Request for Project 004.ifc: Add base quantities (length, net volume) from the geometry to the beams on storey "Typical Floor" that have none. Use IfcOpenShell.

First a look at what the model holds.

```python
import ifcopenshell
import ifcopenshell.util.element
import ifcopenshell.util.unit

model = ifcopenshell.open("Project 004.ifc")
print(model.schema)
for unit_type in ("LENGTHUNIT", "AREAUNIT", "VOLUMEUNIT"):
    print(unit_type, ifcopenshell.util.unit.calculate_unit_scale(model, unit_type))
storey = next(s for s in model.by_type("IfcBuildingStorey") if s.Name == "Typical Floor")
beams = [e for e in ifcopenshell.util.element.get_decomposition(storey) if e.is_a("IfcBeam")]
for e in sorted(beams, key=lambda e: e.id()):
    print(e.id(), e.is_a(), e.Name, list(ifcopenshell.util.element.get_psets(e, qtos_only=True)), sep=" | ")
```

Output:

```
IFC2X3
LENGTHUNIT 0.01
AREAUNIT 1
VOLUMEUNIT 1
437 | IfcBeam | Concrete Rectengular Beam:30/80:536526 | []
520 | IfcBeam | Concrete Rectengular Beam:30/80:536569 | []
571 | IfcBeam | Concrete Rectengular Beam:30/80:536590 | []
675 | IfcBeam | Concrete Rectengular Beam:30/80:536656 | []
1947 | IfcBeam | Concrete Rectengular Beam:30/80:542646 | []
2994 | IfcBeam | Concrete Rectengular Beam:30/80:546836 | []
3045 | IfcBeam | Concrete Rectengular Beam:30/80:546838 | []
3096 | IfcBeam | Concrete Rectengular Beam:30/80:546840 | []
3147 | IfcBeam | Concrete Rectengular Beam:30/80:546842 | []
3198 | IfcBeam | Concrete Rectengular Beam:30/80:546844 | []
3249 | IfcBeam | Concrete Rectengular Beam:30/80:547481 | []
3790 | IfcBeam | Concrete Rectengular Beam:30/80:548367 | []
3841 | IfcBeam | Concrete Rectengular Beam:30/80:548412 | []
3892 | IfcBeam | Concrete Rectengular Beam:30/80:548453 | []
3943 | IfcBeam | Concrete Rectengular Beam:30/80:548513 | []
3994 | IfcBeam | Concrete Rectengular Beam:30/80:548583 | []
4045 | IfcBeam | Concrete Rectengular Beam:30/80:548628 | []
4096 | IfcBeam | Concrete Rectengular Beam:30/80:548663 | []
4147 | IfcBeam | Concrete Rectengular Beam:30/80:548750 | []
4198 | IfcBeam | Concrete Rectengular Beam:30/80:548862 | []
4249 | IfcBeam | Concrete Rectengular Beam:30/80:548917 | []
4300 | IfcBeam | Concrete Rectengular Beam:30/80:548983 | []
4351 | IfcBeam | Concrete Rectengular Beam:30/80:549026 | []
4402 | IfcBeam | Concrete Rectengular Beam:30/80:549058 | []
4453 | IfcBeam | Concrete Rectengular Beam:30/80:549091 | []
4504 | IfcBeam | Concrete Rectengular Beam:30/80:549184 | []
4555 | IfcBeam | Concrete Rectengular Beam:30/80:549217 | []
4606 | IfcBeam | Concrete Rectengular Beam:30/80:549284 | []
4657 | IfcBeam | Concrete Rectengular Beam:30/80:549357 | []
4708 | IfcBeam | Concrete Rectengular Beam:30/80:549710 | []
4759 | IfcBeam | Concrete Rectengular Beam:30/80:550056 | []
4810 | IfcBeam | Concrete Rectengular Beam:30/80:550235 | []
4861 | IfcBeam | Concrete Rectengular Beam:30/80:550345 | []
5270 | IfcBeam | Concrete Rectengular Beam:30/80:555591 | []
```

```python
import ifcopenshell
import ifcopenshell.api.pset
import ifcopenshell.geom
import ifcopenshell.util.element
import ifcopenshell.util.shape
import ifcopenshell.util.unit

model = ifcopenshell.open("Project 004.ifc")
unit_scale = ifcopenshell.util.unit.calculate_unit_scale(model)
volume_scale = ifcopenshell.util.unit.calculate_unit_scale(model, "VOLUMEUNIT")
settings = ifcopenshell.geom.settings()

storey = next(s for s in model.by_type("IfcBuildingStorey") if s.Name == "Typical Floor")
beams = [e for e in ifcopenshell.util.element.get_decomposition(storey) if e.is_a("IfcBeam")]

for e in sorted(beams, key=lambda e: e.id()):
    if ifcopenshell.util.element.get_psets(e, qtos_only=True, should_inherit=False):
        continue
    # Geometry comes back in metres, in the element's own axes.
    shape = ifcopenshell.geom.create_shape(settings, e)
    values = {
        "Length": ifcopenshell.util.shape.get_max_xyz(shape.geometry) / unit_scale,
        "NetVolume": ifcopenshell.util.shape.get_volume(shape.geometry) / volume_scale,
    }
    qto = ifcopenshell.api.pset.add_qto(model, product=e, name="BaseQuantities")
    ifcopenshell.api.pset.edit_qto(model, qto=qto, properties=values)
    print(e.id(), {k: round(v, 3) for k, v in values.items()})

model.write("Project 004_v2.ifc")
```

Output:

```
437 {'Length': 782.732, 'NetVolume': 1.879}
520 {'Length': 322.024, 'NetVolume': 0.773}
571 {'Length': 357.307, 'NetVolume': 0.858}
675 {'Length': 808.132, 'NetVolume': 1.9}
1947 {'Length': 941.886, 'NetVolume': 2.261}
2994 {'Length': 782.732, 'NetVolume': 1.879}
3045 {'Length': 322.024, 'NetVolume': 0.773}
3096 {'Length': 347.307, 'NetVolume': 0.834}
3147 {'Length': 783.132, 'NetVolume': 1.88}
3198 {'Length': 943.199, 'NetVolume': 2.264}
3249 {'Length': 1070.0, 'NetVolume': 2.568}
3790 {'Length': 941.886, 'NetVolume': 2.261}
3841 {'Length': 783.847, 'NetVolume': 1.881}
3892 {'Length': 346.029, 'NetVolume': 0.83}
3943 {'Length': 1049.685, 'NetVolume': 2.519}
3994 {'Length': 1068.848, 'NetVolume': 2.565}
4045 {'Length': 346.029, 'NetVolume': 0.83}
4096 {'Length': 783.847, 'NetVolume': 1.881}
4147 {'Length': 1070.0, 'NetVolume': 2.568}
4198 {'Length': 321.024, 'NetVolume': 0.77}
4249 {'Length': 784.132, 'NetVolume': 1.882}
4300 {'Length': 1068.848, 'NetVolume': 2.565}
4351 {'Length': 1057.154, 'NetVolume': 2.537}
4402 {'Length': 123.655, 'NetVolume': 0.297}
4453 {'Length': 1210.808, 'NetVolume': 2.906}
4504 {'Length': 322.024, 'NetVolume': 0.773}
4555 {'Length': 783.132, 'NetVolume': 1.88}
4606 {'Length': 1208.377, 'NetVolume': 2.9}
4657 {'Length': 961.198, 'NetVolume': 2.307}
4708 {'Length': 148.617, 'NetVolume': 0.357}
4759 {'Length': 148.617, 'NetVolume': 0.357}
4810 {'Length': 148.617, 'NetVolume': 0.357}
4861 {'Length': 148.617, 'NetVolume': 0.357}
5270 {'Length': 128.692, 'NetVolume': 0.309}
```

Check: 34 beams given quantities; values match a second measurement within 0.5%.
